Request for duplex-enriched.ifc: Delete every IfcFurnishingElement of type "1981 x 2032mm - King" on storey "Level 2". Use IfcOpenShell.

First a look at what the model holds.

```python
import ifcopenshell
import ifcopenshell.util.element

model = ifcopenshell.open("duplex-enriched.ifc")
print(model.schema)
storey = next(s for s in model.by_type("IfcBuildingStorey") if s.Name == "Level 2")
furniture = [e for e in ifcopenshell.util.element.get_decomposition(storey) if e.is_a("IfcFurnishingElement")]
seen = {}
for e in furniture:
    element_type = ifcopenshell.util.element.get_type(e)
    name = element_type.Name if element_type not in (None, e) else None
    seen[name] = seen.get(name, 0) + 1
for name, count in sorted(seen.items(), key=str):
    print(count, "x", name)
```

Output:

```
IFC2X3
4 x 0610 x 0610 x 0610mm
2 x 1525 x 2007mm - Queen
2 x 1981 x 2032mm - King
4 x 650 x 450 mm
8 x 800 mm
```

```python
import ifcopenshell
import ifcopenshell.api.root
import ifcopenshell.util.element

model = ifcopenshell.open("duplex-enriched.ifc")

storey = next(s for s in model.by_type("IfcBuildingStorey") if s.Name == "Level 2")
furniture = [e for e in ifcopenshell.util.element.get_decomposition(storey) if e.is_a("IfcFurnishingElement")]
targets = [e for e in furniture if (t := ifcopenshell.util.element.get_type(e)) not in (None, e) and t.Name == "1981 x 2032mm - King"]

for e in targets:
    ifcopenshell.api.root.remove_product(model, product=e)
print(len(targets), "removed")

model.write("duplex-enriched-out.ifc")
```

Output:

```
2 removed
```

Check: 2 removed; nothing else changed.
